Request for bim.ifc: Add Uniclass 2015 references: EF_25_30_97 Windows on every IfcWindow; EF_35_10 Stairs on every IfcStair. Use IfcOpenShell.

First a look at what the model holds.

```python
import ifcopenshell

model = ifcopenshell.open("bim.ifc")
print(model.schema)
print("classifications:", [c.Name for c in model.by_type("IfcClassification")])
for ifc_class in ("IfcDoor", "IfcRoof", "IfcStair", "IfcWall", "IfcWindow"):
    print(ifc_class, len(model.by_type(ifc_class)))
```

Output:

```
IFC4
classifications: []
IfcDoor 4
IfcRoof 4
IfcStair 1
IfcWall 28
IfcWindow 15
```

```python
import ifcopenshell
import ifcopenshell.api.classification

model = ifcopenshell.open("bim.ifc")

system = ifcopenshell.api.classification.add_classification(model, classification="Uniclass 2015")

codes = {
    "IfcWindow": ("EF_25_30_97", "Windows"),
    "IfcStair": ("EF_35_10", "Stairs"),
}
for ifc_class, (code, name) in codes.items():
    products = model.by_type(ifc_class)
    ifcopenshell.api.classification.add_reference(
        model, products=products, classification=system, identification=code, name=name
    )
    print(code, len(products))

model.write("bim_edited.ifc")
```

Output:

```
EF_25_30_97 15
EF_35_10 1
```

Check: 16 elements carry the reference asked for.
